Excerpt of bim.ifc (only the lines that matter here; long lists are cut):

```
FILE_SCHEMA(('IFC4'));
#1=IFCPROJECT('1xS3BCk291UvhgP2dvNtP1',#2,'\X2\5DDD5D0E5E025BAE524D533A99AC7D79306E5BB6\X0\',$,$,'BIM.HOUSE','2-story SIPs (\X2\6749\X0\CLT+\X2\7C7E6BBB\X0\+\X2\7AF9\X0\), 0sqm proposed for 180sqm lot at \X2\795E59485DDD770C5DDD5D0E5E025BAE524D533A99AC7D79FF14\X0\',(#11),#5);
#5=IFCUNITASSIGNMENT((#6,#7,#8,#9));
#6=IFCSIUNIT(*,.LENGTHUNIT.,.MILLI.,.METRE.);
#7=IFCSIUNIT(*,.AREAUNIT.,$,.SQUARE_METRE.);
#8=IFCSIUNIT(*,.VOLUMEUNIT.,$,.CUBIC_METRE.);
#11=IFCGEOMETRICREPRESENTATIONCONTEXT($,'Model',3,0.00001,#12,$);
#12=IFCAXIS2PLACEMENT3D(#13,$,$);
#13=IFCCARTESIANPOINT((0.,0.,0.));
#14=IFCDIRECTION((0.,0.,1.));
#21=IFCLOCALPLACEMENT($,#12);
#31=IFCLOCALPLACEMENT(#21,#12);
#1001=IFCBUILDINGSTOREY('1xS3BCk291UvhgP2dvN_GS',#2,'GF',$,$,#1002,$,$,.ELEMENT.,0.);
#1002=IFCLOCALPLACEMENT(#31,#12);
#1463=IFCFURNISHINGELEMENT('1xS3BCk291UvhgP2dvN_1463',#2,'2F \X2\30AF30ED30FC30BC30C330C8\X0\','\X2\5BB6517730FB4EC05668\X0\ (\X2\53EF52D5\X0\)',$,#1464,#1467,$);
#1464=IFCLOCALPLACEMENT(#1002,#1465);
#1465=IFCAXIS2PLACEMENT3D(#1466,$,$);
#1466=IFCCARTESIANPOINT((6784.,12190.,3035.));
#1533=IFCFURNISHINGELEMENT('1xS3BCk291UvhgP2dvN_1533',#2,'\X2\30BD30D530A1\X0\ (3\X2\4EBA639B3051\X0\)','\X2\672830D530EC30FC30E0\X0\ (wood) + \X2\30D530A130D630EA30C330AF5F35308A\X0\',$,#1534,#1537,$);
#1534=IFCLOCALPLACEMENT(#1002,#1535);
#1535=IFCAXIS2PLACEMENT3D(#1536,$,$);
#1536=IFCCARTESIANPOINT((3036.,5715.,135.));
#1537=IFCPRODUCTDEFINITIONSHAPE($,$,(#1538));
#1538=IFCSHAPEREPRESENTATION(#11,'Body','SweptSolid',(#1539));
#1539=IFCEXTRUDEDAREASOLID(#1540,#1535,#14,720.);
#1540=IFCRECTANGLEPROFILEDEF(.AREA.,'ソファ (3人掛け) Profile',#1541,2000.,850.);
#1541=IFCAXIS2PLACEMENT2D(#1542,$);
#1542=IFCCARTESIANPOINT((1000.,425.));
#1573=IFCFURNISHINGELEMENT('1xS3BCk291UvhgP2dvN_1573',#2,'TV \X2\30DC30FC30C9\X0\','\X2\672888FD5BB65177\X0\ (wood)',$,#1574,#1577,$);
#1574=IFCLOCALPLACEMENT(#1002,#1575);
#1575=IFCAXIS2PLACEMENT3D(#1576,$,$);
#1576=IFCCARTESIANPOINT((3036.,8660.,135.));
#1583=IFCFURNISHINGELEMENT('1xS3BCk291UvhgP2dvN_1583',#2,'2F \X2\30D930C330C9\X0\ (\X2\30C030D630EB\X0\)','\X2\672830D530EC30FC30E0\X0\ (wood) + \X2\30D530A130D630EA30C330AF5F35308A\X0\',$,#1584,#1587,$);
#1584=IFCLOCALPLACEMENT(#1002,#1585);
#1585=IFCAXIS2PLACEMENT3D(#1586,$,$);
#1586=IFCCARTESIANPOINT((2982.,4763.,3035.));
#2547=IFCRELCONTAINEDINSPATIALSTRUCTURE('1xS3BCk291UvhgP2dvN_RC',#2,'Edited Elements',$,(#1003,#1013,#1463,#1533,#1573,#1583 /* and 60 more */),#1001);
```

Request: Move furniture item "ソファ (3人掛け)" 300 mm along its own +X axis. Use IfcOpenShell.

```python
import ifcopenshell
import ifcopenshell.api.geometry
import ifcopenshell.util.placement
import ifcopenshell.util.unit

model = ifcopenshell.open("bim.ifc")
unit_scale = ifcopenshell.util.unit.calculate_unit_scale(model)

item = model.by_guid("1xS3BCk291UvhgP2dvN_1533")
matrix = ifcopenshell.util.placement.get_local_placement(item.ObjectPlacement)
matrix[:3, 3] += matrix[:3, 0] * 0.3 / unit_scale
ifcopenshell.api.geometry.edit_object_placement(model, product=item, matrix=matrix, is_si=False)

print(ifcopenshell.util.placement.get_local_placement(item.ObjectPlacement).round(3) + 0.0)

model.write("bim_edited.ifc")
```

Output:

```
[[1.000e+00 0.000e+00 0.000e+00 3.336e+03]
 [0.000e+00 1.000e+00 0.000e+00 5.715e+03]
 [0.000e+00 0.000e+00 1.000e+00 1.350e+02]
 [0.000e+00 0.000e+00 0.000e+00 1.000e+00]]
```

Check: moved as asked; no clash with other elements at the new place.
